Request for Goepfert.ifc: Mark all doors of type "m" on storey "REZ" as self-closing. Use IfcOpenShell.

First a look at what the model holds.

```python
import ifcopenshell
import ifcopenshell.util.element

model = ifcopenshell.open("Goepfert.ifc")
print(model.schema)
storey = next(s for s in model.by_type("IfcBuildingStorey") if s.Name == "REZ")
doors = [e for e in ifcopenshell.util.element.get_decomposition(storey) if e.is_a("IfcDoor")]
seen = {}
for e in doors:
    element_type = ifcopenshell.util.element.get_type(e)
    key = (element_type.Name if element_type != e and element_type else None, ifcopenshell.util.element.get_pset(e, "Pset_DoorCommon", "SelfClosing"))
    seen[key] = seen.get(key, 0) + 1
for (name, value), count in sorted(seen.items(), key=str):
    print(count, "x", name, "|", value)
```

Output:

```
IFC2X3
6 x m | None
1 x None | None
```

```python
import ifcopenshell
import ifcopenshell.api.pset
import ifcopenshell.util.element

model = ifcopenshell.open("Goepfert.ifc")

storey = next(s for s in model.by_type("IfcBuildingStorey") if s.Name == "REZ")
doors = [e for e in ifcopenshell.util.element.get_decomposition(storey) if e.is_a("IfcDoor")]

count = 0
for e in doors:
    element_type = ifcopenshell.util.element.get_type(e)
    if element_type in (None, e) or element_type.Name != "m":
        continue
    # add_pset returns the element's existing set when there is one.
    pset = ifcopenshell.api.pset.add_pset(model, product=e, name="Pset_DoorCommon")
    ifcopenshell.api.pset.edit_pset(model, pset=pset, properties={"SelfClosing": True})
    count += 1

print(count, "doors updated")

model.write("Goepfert_updated.ifc")
```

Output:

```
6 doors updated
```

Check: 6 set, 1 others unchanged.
